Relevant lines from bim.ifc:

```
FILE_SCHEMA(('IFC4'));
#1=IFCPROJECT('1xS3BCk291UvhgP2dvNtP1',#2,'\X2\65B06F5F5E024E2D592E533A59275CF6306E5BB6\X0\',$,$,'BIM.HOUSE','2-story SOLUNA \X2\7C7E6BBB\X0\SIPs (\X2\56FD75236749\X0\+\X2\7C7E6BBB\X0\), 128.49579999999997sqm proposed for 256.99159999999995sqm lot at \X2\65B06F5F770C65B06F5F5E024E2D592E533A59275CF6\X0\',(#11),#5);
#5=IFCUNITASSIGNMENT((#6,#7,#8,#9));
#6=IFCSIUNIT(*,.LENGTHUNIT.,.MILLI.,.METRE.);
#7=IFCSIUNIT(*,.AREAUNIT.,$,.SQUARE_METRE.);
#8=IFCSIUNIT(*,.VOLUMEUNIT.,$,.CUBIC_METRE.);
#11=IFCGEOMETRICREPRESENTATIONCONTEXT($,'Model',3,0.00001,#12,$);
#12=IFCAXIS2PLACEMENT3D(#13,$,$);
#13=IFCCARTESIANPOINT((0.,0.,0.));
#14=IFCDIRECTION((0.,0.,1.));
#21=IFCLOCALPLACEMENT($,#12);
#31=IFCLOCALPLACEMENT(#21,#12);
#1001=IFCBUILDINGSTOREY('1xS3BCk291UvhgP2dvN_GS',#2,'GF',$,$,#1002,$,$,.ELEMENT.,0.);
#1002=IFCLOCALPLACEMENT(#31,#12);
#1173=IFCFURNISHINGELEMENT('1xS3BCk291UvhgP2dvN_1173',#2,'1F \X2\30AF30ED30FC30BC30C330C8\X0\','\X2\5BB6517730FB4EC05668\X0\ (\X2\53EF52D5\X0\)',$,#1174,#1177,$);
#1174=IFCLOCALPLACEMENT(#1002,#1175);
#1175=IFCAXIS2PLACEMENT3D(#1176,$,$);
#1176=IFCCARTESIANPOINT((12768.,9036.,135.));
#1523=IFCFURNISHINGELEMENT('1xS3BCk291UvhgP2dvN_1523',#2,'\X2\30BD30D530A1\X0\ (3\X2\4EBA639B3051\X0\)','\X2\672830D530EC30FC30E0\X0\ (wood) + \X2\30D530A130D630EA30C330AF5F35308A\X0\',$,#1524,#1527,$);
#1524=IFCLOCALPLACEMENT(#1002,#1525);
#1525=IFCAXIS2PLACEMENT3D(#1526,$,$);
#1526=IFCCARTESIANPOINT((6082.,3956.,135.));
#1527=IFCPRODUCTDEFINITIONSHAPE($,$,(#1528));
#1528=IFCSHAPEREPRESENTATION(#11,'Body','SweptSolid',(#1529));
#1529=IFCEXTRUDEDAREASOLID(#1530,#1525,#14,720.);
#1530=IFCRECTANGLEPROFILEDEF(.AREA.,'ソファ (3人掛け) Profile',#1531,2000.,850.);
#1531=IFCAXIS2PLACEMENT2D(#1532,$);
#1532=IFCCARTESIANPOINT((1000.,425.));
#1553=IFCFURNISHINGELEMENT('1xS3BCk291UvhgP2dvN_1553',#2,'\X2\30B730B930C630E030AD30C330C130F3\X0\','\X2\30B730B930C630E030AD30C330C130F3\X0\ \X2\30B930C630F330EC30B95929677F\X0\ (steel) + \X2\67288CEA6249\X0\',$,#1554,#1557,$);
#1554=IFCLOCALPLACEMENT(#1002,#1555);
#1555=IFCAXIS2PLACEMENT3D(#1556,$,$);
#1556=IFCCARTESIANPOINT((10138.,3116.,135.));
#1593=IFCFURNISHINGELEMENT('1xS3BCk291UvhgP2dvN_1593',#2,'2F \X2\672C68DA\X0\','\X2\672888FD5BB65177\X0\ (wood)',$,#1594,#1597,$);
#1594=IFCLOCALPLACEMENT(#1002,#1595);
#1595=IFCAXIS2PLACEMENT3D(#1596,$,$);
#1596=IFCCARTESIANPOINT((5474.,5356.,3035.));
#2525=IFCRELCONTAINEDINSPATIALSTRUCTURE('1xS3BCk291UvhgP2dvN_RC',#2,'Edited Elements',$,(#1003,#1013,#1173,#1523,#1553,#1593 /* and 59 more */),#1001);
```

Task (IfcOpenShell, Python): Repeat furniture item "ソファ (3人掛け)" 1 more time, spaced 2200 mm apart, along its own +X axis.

```python
import ifcopenshell
import ifcopenshell.api.geometry
import ifcopenshell.api.root
import ifcopenshell.util.element
import ifcopenshell.util.placement

model = ifcopenshell.open("bim.ifc")


def reuse_history(source, copy):
    """copy_class also copies each property set's owner history, people and application; keep the originals."""
    for rel in copy.IsDefinedBy:
        if rel.is_a("IfcRelDefinesByProperties") and (history := rel.RelatingPropertyDefinition.OwnerHistory):
            rel.RelatingPropertyDefinition.OwnerHistory = source.OwnerHistory
            ifcopenshell.util.element.remove_deep2(model, history)


source = model.by_id(1523)
base = ifcopenshell.util.placement.get_local_placement(source.ObjectPlacement)
step = base[:3, 0] * 2200.0

for i in range(1, 2):
    copy = ifcopenshell.api.root.copy_class(model, product=source)
    copy.Representation = ifcopenshell.util.element.copy_deep(
        model, source.Representation, exclude=["IfcGeometricRepresentationContext", "IfcRepresentationMap"]
    )
    reuse_history(source, copy)
    matrix = base.copy()
    matrix[:3, 3] += i * step
    print("added at", matrix[:3, 3].round(3) + 0.0)
    ifcopenshell.api.geometry.edit_object_placement(model, product=copy, matrix=matrix, is_si=False)

model.write("bim-out.ifc")
```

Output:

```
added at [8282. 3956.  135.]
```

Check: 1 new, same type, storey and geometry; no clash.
